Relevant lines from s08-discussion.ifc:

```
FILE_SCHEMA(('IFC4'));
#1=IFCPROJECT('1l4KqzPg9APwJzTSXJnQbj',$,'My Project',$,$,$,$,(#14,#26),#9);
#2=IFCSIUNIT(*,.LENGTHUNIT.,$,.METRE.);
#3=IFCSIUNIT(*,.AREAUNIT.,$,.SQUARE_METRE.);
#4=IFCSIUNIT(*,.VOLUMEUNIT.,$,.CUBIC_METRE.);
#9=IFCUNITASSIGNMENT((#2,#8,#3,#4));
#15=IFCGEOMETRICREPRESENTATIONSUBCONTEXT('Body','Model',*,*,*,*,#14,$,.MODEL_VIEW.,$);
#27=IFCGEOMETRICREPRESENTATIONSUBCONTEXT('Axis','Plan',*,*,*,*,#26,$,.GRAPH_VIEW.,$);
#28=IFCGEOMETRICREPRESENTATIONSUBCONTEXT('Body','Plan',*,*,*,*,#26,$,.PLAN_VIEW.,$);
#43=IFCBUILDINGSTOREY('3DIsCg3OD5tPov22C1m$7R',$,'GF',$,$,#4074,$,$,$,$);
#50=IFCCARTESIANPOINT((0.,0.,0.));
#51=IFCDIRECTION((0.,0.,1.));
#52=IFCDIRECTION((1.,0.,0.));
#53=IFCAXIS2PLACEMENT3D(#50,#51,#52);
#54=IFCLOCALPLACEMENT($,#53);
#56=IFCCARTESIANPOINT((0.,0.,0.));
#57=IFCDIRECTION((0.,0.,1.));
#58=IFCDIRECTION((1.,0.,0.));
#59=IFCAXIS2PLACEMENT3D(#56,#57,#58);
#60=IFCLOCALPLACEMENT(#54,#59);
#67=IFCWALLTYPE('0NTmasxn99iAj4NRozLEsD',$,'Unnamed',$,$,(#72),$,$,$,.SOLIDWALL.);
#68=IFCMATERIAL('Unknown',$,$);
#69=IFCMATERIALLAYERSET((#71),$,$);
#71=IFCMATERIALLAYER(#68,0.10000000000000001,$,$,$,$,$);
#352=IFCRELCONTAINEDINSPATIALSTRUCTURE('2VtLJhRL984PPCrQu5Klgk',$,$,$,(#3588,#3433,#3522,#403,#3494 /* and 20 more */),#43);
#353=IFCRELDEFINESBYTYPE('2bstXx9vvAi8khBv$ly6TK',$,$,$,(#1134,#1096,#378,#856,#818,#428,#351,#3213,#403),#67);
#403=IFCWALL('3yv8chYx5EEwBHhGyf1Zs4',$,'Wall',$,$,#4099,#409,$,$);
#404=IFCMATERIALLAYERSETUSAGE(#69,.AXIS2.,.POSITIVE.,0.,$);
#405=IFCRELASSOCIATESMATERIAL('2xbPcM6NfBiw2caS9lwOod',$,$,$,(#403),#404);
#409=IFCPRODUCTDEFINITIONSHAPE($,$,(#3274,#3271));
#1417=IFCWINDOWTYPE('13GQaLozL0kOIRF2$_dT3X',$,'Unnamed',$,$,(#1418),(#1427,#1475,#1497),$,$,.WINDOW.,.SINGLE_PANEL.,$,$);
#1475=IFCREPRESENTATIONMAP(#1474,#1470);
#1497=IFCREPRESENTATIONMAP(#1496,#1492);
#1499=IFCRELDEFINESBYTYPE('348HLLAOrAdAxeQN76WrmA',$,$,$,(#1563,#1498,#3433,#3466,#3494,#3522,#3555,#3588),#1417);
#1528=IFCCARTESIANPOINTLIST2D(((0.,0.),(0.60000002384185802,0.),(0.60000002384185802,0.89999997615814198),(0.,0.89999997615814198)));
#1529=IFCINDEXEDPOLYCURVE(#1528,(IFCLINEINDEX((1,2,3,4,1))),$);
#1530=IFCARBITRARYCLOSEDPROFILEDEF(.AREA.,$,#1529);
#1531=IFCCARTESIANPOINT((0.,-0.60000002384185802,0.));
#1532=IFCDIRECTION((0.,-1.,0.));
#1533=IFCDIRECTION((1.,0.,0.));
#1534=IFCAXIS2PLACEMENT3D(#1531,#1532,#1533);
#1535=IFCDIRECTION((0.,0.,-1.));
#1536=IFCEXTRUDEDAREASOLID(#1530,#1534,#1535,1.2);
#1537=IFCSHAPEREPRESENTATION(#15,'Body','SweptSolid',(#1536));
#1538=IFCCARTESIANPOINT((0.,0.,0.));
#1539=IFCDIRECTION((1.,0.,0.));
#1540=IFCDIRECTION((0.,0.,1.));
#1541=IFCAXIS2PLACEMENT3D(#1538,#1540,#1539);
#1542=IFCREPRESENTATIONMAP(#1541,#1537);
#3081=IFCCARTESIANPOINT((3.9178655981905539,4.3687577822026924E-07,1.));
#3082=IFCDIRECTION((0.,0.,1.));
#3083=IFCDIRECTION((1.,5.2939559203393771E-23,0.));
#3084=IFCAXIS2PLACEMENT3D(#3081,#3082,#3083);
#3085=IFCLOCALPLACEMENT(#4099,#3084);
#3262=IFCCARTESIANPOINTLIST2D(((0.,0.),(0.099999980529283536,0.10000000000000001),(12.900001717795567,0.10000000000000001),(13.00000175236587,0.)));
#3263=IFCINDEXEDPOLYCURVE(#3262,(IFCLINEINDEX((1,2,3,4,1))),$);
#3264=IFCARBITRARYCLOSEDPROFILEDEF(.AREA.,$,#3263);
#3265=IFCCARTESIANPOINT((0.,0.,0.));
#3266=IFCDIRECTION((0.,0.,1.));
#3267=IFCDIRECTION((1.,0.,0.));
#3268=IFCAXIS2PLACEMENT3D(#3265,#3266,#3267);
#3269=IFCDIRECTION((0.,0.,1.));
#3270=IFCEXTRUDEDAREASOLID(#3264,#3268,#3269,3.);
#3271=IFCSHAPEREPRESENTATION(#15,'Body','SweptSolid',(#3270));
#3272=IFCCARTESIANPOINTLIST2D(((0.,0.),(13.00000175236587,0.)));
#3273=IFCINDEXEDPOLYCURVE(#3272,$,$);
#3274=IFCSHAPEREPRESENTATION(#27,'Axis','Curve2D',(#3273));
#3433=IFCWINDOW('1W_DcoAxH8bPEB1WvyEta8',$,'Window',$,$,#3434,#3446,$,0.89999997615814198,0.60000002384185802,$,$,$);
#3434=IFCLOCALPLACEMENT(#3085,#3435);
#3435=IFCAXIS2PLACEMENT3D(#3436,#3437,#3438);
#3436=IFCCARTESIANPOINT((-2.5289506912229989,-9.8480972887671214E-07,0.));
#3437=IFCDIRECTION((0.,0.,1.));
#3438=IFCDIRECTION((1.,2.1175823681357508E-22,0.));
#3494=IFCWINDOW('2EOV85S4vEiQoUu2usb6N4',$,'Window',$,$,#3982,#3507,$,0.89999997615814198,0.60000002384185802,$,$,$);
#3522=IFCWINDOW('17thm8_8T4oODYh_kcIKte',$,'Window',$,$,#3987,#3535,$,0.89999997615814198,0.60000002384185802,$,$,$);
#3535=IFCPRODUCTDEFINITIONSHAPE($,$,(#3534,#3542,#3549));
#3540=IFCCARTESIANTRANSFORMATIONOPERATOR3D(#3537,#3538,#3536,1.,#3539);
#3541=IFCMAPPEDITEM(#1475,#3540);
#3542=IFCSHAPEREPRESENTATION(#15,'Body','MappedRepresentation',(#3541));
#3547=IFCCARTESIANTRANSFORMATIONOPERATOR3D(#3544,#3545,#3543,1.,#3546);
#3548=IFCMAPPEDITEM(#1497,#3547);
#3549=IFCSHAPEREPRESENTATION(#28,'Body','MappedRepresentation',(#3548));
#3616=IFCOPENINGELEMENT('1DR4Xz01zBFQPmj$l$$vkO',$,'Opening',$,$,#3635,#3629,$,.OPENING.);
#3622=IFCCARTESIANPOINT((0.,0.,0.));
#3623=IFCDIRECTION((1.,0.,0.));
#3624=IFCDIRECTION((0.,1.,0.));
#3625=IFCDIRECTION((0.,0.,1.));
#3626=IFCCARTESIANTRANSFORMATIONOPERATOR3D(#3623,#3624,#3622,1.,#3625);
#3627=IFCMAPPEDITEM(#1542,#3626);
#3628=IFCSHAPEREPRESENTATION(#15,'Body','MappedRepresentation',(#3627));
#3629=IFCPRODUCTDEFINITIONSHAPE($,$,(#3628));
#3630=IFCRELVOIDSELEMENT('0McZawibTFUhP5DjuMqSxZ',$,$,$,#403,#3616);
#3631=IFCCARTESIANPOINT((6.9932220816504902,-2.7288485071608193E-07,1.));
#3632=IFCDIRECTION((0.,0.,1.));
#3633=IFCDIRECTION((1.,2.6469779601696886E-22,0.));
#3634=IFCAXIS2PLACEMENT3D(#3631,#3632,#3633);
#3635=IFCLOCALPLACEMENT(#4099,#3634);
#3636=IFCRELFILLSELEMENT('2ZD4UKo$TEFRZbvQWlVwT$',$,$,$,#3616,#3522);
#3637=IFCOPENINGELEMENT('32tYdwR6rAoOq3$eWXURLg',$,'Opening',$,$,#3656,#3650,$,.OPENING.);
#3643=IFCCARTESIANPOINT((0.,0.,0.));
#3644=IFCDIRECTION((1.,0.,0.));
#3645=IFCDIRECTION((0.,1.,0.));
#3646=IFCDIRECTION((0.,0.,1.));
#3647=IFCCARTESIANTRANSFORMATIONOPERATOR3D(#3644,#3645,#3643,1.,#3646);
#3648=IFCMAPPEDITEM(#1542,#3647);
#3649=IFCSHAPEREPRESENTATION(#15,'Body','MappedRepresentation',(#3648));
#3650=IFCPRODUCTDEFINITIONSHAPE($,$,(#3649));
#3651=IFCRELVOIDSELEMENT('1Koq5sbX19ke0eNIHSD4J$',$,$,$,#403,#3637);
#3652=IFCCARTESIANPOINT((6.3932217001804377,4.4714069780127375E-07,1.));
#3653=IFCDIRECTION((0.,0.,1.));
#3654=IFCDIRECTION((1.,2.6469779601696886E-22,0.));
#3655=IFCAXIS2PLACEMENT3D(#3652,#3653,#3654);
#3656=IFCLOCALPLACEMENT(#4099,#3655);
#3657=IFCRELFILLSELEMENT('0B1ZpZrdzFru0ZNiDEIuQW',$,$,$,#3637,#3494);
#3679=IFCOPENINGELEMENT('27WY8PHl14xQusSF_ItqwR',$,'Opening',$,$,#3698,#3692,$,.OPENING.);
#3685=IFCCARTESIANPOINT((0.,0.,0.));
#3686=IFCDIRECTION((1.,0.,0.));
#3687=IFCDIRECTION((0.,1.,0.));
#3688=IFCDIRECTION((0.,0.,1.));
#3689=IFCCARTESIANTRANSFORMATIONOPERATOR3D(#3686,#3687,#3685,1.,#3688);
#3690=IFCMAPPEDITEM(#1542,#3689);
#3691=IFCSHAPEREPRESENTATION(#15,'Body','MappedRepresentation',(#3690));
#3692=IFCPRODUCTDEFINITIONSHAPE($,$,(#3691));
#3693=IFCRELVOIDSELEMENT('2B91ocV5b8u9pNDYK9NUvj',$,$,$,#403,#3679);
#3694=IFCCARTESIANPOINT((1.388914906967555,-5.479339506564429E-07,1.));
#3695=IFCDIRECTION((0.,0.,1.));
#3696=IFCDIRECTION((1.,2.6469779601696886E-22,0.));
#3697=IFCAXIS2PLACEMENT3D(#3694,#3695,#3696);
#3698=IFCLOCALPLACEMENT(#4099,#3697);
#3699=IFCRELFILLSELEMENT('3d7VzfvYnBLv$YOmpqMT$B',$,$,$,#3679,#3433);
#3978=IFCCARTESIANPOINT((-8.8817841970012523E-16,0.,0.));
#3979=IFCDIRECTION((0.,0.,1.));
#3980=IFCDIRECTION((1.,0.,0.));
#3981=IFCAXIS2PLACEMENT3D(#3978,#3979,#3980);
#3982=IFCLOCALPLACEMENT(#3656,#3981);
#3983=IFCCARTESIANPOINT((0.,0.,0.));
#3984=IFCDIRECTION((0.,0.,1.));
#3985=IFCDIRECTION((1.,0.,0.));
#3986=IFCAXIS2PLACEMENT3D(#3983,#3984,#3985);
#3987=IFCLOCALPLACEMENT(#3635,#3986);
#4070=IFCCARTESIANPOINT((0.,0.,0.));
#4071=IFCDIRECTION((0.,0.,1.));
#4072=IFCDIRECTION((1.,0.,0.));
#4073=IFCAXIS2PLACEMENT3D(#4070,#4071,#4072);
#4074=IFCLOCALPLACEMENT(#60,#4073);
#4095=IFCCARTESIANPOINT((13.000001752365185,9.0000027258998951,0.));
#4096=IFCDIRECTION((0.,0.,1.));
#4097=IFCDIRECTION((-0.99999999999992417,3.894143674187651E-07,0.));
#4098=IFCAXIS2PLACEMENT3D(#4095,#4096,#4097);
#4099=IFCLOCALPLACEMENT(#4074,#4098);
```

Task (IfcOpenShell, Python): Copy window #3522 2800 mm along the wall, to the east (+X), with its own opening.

```python
import ifcopenshell
import ifcopenshell.api.feature
import ifcopenshell.api.geometry
import ifcopenshell.api.root
import ifcopenshell.geom
import ifcopenshell.util.element
import ifcopenshell.util.placement
import ifcopenshell.util.shape
import ifcopenshell.util.unit

model = ifcopenshell.open("s08-discussion.ifc")
unit_scale = ifcopenshell.util.unit.calculate_unit_scale(model)
settings = ifcopenshell.geom.settings()


def volume(element):
    """Net volume in cubic metres, openings subtracted."""
    shape = ifcopenshell.geom.create_shape(settings, element)
    return ifcopenshell.util.shape.get_volume(shape.geometry)


window = model.by_id(3522)
opening = window.FillsVoids[0].RelatingOpeningElement
wall = opening.VoidsElements[0].RelatingBuildingElement
before = volume(wall)
shift = ifcopenshell.util.placement.get_local_placement(wall.ObjectPlacement)[:3, 0] * -2.8 / unit_scale

# copy_class copies the void relationship, type, container and properties, but no geometry.
new_opening = ifcopenshell.api.root.copy_class(model, product=opening)
new_opening.Representation = ifcopenshell.util.element.copy_deep(
    model, opening.Representation, exclude=["IfcGeometricRepresentationContext", "IfcRepresentationMap"]
)
new_window = ifcopenshell.api.root.copy_class(model, product=window)
new_window.Representation = ifcopenshell.util.element.copy_deep(
    model, window.Representation, exclude=["IfcGeometricRepresentationContext", "IfcRepresentationMap"]
)
ifcopenshell.api.feature.add_filling(model, opening=new_opening, element=new_window)

for old, new in ((opening, new_opening), (window, new_window)):
    matrix = ifcopenshell.util.placement.get_local_placement(old.ObjectPlacement)
    matrix[:3, 3] += shift
    ifcopenshell.api.geometry.edit_object_placement(model, product=new, matrix=matrix, is_si=False)

after = volume(wall)

print(f"wall volume {before:.3f} -> {after:.3f} m3")

model.write("s08-discussion_updated.ifc")
```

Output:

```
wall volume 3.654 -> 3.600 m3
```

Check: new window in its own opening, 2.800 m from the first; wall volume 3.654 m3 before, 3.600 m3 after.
